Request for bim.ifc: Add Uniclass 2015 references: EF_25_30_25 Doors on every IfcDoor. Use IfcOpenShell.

First a look at what the model holds.

```python
import ifcopenshell

model = ifcopenshell.open("bim.ifc")
print(model.schema)
print("classifications:", [c.Name for c in model.by_type("IfcClassification")])
for ifc_class in ("IfcDoor", "IfcRoof", "IfcStair", "IfcWall", "IfcWindow"):
    print(ifc_class, len(model.by_type(ifc_class)))
```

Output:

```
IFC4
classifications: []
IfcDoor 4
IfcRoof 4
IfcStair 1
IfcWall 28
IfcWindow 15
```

```python
import ifcopenshell
import ifcopenshell.api.classification

model = ifcopenshell.open("bim.ifc")

system = ifcopenshell.api.classification.add_classification(model, classification="Uniclass 2015")

codes = {
    "IfcDoor": ("EF_25_30_25", "Doors"),
}
for ifc_class, (code, name) in codes.items():
    products = model.by_type(ifc_class)
    ifcopenshell.api.classification.add_reference(
        model, products=products, classification=system, identification=code, name=name
    )
    print(code, len(products))

model.write("bim_rev.ifc")
```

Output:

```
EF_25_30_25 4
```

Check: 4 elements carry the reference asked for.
